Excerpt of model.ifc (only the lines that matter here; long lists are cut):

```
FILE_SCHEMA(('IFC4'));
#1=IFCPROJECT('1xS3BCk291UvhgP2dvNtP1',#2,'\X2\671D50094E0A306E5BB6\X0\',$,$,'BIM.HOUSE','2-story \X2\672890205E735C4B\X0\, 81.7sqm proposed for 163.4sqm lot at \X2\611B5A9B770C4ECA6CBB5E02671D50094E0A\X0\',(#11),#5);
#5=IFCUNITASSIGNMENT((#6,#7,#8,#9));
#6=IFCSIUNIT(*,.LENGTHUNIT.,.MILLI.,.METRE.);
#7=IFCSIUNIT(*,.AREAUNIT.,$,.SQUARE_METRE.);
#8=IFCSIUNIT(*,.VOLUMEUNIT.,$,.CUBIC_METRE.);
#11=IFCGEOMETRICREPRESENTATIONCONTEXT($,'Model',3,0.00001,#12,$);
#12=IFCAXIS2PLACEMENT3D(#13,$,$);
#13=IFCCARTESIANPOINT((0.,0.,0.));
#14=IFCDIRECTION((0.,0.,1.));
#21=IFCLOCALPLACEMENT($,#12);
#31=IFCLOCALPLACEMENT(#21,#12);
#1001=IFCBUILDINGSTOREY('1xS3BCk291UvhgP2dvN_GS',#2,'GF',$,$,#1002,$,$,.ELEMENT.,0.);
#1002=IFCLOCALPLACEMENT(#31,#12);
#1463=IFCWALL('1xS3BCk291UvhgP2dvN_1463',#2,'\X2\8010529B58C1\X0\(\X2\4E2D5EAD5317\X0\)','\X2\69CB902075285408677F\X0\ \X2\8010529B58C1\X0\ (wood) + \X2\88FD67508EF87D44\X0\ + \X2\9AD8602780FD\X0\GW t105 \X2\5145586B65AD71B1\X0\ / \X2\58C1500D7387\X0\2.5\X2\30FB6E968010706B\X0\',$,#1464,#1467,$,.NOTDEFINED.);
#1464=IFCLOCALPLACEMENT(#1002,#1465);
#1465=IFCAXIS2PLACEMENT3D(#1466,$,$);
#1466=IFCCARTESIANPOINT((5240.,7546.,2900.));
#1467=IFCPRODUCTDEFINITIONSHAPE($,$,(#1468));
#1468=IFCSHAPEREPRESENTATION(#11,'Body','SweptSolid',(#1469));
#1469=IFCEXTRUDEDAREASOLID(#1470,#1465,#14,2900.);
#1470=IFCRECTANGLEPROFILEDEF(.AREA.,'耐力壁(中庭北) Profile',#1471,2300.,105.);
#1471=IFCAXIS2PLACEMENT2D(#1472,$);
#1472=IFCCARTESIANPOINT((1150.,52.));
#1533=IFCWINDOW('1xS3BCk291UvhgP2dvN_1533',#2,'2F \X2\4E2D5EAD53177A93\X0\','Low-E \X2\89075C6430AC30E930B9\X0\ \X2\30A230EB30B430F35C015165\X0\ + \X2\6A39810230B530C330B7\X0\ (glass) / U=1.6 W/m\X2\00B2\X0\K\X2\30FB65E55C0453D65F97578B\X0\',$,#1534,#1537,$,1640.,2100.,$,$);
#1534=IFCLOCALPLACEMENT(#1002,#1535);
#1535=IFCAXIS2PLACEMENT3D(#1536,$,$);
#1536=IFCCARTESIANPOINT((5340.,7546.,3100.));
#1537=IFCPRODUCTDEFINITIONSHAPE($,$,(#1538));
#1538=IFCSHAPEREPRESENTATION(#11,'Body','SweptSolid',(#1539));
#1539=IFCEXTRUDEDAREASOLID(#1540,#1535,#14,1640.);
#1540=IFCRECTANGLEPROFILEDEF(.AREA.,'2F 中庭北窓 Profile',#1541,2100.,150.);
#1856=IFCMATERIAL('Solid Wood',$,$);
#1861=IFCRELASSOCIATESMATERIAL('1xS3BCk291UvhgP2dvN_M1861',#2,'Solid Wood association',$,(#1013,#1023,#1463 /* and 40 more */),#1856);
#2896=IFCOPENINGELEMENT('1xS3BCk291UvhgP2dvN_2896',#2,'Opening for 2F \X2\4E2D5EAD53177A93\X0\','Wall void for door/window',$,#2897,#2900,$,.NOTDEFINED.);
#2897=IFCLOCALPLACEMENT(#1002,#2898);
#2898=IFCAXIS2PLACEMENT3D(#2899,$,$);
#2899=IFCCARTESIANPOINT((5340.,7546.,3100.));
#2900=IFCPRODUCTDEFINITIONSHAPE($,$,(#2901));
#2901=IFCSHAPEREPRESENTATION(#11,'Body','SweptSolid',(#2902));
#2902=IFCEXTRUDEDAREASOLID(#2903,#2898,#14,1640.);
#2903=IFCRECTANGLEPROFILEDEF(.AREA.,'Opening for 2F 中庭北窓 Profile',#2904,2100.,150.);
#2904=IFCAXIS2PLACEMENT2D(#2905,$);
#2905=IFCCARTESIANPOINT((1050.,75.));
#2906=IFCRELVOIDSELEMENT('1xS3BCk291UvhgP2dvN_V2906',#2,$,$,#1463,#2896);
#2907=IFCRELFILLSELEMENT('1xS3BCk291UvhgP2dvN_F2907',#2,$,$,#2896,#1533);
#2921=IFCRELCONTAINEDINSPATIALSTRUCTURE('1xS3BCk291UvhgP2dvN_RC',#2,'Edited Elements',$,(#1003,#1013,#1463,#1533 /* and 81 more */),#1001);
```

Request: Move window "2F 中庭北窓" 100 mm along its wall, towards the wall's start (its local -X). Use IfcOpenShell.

```python
import ifcopenshell
import ifcopenshell.api.geometry
import ifcopenshell.util.placement

model = ifcopenshell.open("model.ifc")

window = model.by_guid("1xS3BCk291UvhgP2dvN_1533")
opening = window.FillsVoids[0].RelatingOpeningElement
wall = opening.VoidsElements[0].RelatingBuildingElement

wall_matrix = ifcopenshell.util.placement.get_local_placement(wall.ObjectPlacement)
shift = wall_matrix[:3, 0] * -100.0
before = ifcopenshell.util.placement.get_local_placement(window.ObjectPlacement)[:3, 3].copy()

# The window is not placed relative to its opening, so move both.
for product in (opening, window):
    matrix = ifcopenshell.util.placement.get_local_placement(product.ObjectPlacement)
    matrix[:3, 3] += shift
    ifcopenshell.api.geometry.edit_object_placement(model, product=product, matrix=matrix, is_si=False)

after = ifcopenshell.util.placement.get_local_placement(window.ObjectPlacement)[:3, 3]
print("window moved by", (after - before).round(3) + 0.0)

model.write("model_updated.ifc")
```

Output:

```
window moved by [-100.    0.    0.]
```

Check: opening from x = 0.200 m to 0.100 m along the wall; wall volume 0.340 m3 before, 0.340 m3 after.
